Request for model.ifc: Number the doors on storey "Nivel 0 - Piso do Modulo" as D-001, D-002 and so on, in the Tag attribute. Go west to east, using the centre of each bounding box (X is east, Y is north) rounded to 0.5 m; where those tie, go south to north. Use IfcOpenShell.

First a look at what the model holds.

```python
import ifcopenshell
import ifcopenshell.util.element
import ifcopenshell.util.placement

model = ifcopenshell.open("model.ifc")
print(model.schema)
storey = next(s for s in model.by_type("IfcBuildingStorey") if s.Name == "Nivel 0 - Piso do Modulo")
doors = [e for e in ifcopenshell.util.element.get_decomposition(storey) if e.is_a("IfcDoor")]
for e in sorted(doors, key=lambda e: e.id()):
    origin = ifcopenshell.util.placement.get_local_placement(e.ObjectPlacement)[:3, 3]
    print(e.id(), e.Tag, e.Name, origin.round(2) + 0.0, sep=" | ")
```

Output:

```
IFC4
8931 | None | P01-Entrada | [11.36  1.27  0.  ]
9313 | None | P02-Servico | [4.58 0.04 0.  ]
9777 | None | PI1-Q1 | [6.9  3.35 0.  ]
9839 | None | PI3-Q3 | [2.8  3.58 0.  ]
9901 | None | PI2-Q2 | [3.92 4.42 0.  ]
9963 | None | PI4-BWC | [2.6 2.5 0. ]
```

```python
import ifcopenshell
import ifcopenshell.geom
import ifcopenshell.util.element
import ifcopenshell.util.shape

model = ifcopenshell.open("model.ifc")
settings = ifcopenshell.geom.settings()
settings.set("use-world-coords", True)


def centre(element):
    shape = ifcopenshell.geom.create_shape(settings, element)
    return ifcopenshell.util.shape.get_bbox_centroid(shape.geometry)


storey = next(s for s in model.by_type("IfcBuildingStorey") if s.Name == "Nivel 0 - Piso do Modulo")
doors = [e for e in ifcopenshell.util.element.get_decomposition(storey) if e.is_a("IfcDoor")]

# Insertion points can sit at a corner or the storey origin, so sort by the geometry (in metres).
centres = {e: centre(e) for e in doors}
doors.sort(key=lambda e: (round(centres[e][0] / 0.5), centres[e][1]))

for i, e in enumerate(doors, start=1):
    number = f"D-0{i:02d}"
    e.Tag = number
    print(e.id(), number)

model.write("model_edited.ifc")
```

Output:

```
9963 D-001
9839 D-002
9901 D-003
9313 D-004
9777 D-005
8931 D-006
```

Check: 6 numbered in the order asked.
